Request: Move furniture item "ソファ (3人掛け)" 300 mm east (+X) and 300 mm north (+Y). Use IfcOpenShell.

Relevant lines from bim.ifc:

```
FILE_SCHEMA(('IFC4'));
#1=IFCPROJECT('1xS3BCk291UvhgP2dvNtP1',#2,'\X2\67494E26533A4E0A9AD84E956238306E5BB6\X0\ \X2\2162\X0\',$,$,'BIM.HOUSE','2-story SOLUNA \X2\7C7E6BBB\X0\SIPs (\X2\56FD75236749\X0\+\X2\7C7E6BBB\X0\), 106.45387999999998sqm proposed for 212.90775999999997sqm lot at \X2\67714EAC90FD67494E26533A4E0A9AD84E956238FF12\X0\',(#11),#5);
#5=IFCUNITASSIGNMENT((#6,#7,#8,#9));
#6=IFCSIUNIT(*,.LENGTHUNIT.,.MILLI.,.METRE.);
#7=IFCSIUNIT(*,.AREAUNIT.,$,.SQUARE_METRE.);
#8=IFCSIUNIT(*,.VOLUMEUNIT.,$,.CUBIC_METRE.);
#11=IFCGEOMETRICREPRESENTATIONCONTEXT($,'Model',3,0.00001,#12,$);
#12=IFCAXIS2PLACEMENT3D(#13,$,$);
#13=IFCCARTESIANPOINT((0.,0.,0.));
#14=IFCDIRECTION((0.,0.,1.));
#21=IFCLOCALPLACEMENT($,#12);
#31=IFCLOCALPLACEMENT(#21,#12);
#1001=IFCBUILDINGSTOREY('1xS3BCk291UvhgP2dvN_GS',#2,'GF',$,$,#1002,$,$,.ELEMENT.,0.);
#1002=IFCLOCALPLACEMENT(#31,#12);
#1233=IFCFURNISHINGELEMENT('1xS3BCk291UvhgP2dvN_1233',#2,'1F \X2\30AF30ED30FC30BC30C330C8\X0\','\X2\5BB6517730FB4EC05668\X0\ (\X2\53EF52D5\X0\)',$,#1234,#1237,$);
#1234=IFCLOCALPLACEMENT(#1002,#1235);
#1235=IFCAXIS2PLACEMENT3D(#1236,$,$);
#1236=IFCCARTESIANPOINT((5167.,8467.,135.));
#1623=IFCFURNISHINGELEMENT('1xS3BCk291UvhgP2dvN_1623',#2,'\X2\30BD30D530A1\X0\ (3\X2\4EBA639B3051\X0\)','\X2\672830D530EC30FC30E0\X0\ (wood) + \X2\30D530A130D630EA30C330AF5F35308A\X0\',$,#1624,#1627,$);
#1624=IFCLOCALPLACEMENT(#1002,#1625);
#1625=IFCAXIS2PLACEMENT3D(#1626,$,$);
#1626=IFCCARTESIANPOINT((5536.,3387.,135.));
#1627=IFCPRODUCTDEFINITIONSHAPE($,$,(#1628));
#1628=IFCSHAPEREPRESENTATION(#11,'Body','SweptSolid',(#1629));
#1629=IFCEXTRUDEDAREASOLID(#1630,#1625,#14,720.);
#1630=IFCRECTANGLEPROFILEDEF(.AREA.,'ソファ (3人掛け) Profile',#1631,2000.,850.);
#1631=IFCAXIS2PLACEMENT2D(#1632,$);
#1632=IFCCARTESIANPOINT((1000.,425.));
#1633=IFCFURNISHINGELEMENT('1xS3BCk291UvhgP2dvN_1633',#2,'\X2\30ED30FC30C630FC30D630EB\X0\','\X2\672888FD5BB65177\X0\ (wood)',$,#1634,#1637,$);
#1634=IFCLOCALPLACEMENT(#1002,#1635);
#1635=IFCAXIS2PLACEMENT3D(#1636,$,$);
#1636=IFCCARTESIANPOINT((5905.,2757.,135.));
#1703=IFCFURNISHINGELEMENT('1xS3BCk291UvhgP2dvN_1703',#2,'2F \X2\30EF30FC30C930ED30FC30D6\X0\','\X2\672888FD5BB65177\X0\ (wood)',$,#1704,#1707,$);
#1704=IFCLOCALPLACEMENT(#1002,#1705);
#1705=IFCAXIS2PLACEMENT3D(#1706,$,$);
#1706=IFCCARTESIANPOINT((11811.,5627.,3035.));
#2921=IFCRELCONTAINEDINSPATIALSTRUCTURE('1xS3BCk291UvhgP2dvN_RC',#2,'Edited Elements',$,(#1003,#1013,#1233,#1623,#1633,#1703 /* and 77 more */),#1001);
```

```python
import ifcopenshell
import ifcopenshell.api.geometry
import ifcopenshell.util.placement

model = ifcopenshell.open("bim.ifc")

item = model.by_id(1623)
matrix = ifcopenshell.util.placement.get_local_placement(item.ObjectPlacement)
matrix[0, 3] += 300.0
matrix[1, 3] += 300.0
ifcopenshell.api.geometry.edit_object_placement(model, product=item, matrix=matrix, is_si=False)

print(ifcopenshell.util.placement.get_local_placement(item.ObjectPlacement).round(3) + 0.0)

model.write("bim-out.ifc")
```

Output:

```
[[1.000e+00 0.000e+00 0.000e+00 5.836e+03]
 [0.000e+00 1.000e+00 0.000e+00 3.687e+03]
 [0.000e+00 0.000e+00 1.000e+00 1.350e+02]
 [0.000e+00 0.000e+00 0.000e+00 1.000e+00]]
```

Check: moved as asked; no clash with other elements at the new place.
